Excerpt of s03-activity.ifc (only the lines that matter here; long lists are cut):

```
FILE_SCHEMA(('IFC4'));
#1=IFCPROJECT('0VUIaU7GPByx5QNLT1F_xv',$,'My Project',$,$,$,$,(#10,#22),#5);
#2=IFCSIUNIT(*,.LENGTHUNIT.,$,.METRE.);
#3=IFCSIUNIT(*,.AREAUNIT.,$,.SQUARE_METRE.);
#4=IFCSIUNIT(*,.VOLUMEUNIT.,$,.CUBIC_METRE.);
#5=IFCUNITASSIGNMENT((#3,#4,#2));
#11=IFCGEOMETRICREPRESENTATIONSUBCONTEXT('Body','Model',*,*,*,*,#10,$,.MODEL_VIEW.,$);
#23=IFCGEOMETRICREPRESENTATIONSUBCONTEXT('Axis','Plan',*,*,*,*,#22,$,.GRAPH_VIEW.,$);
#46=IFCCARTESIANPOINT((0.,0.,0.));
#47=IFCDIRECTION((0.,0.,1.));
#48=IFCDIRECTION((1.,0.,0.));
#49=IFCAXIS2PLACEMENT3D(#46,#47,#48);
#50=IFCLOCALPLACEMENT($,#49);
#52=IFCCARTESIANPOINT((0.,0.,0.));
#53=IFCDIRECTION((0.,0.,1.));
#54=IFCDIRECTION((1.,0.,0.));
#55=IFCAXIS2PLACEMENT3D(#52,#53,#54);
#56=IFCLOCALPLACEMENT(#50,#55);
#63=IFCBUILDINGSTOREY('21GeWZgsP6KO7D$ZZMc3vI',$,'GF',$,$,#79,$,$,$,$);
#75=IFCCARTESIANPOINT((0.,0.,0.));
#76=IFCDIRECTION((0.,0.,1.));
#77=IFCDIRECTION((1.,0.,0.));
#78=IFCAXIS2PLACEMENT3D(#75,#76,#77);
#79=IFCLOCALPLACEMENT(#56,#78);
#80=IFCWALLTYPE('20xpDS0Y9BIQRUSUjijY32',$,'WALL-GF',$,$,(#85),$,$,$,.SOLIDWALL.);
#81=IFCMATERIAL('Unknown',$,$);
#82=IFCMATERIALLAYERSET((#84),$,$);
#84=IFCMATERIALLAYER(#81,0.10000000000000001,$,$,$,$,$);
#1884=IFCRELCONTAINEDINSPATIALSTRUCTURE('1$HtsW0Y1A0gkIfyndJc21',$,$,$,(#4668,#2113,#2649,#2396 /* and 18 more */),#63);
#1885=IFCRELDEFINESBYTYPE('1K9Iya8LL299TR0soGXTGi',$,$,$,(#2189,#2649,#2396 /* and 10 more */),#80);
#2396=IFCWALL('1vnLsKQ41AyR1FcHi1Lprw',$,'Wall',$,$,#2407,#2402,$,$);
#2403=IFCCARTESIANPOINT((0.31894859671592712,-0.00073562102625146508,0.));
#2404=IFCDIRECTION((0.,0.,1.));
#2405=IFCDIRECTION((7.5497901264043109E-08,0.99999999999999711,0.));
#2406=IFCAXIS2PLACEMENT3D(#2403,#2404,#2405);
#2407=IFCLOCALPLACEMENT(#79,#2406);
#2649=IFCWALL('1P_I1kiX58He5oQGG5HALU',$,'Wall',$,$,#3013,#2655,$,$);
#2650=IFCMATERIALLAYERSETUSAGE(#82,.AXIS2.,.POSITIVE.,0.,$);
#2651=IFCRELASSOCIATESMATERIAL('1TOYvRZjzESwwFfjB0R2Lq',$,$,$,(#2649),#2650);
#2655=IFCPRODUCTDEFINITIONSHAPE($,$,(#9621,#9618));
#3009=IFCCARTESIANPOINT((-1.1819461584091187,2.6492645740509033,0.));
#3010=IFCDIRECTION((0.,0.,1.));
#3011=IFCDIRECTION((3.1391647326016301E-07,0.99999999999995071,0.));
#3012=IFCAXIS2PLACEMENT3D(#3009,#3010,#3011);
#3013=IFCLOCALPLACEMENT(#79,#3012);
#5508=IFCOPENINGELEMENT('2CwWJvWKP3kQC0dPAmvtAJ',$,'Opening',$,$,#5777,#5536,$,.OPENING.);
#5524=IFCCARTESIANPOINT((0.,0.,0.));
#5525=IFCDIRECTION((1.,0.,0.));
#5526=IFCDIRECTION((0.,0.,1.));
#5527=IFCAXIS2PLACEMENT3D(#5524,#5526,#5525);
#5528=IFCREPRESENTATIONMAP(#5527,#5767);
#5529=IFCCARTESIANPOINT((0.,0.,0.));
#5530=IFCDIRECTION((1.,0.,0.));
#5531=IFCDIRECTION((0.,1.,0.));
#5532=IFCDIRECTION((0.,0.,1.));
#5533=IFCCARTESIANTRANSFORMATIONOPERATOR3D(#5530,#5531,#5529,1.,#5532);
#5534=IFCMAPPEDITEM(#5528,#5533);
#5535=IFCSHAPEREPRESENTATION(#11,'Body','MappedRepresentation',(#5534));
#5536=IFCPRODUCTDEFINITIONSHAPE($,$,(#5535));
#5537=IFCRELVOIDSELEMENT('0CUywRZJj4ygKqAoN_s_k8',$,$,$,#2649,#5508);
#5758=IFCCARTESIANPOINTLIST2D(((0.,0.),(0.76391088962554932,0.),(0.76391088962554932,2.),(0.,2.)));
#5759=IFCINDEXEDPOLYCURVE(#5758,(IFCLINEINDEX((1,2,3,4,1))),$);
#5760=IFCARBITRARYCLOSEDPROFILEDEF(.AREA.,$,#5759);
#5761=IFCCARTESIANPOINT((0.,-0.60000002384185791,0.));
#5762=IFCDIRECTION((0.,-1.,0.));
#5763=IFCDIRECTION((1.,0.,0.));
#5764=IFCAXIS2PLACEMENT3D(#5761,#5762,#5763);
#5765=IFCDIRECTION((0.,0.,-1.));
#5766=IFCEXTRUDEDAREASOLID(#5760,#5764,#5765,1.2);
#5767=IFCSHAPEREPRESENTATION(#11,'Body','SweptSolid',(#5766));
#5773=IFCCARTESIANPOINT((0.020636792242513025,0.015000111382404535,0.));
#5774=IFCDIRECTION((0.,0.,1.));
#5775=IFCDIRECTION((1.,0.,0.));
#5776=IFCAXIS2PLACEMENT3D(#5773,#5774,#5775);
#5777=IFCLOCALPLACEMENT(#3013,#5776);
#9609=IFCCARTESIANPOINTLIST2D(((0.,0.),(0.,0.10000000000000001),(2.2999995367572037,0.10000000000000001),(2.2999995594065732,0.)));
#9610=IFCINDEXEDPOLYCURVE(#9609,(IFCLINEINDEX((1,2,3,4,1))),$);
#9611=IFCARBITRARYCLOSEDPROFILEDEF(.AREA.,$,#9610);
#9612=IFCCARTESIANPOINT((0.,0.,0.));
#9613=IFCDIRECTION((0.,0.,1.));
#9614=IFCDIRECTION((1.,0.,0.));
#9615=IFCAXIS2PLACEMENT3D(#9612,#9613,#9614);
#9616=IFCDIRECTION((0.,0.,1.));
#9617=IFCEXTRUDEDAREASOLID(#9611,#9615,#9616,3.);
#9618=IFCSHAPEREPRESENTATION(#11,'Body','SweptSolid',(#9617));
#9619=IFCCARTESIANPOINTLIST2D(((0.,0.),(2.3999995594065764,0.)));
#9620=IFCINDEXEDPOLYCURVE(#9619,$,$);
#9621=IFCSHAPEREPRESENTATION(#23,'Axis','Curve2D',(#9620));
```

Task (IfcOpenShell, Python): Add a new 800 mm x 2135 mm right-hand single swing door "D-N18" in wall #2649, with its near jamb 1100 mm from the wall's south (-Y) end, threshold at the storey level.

```python
import numpy as np
import ifcopenshell
import ifcopenshell.api.feature
import ifcopenshell.api.geometry
import ifcopenshell.api.root
import ifcopenshell.api.spatial
import ifcopenshell.geom
import ifcopenshell.util.element
import ifcopenshell.util.placement
import ifcopenshell.util.representation
import ifcopenshell.util.shape
import ifcopenshell.util.unit

model = ifcopenshell.open("s03-activity.ifc")
unit_scale = ifcopenshell.util.unit.calculate_unit_scale(model)
settings = ifcopenshell.geom.settings()


def volume(element):
    """Net volume in cubic metres, openings subtracted."""
    shape = ifcopenshell.geom.create_shape(settings, element)
    return ifcopenshell.util.shape.get_volume(shape.geometry)


wall = model.by_guid("1P_I1kiX58He5oQGG5HALU")
storey = ifcopenshell.util.element.get_container(wall, ifc_class="IfcBuildingStorey")
context = ifcopenshell.util.representation.get_context(model, "Model", "Body", "MODEL_VIEW")
before = volume(wall)

width, height, from_end, sill = 0.8, 2.135, 1.1, 0.0  # metres

# The wall runs along its own X axis, and the end named is its -X end.
wall_shape = ifcopenshell.geom.create_shape(settings, wall)
x, y, z = ifcopenshell.util.shape.get_vertices(wall_shape.geometry).T
start = x.min() + from_end
face, thickness = float(y.min()), float(y.max() - y.min())
wall_matrix = ifcopenshell.util.placement.get_local_placement(wall.ObjectPlacement)
level = ifcopenshell.util.placement.get_local_placement(storey.ObjectPlacement)[2, 3]


def in_wall(x, y):
    """Placement at x, y metres in the wall's axes, at sill height."""
    matrix = wall_matrix.copy()
    matrix[:, 3] = wall_matrix @ np.array([x / unit_scale, y / unit_scale, 0.0, 1.0])
    matrix[2, 3] = level + sill / unit_scale
    return matrix


# Opening: a box that overshoots both wall faces by 50 mm.
opening = ifcopenshell.api.root.create_entity(model, ifc_class="IfcOpeningElement", predefined_type="OPENING")
box = ifcopenshell.api.geometry.add_wall_representation(
    model, context=context, length=width, height=height, thickness=thickness + 0.1
)
ifcopenshell.api.geometry.assign_representation(model, product=opening, representation=box)
ifcopenshell.api.geometry.edit_object_placement(model, product=opening, matrix=in_wall(start, face - 0.05), is_si=False)
ifcopenshell.api.feature.add_feature(model, feature=opening, element=wall)

door = ifcopenshell.api.root.create_entity(model, ifc_class="IfcDoor", name="D-N18", predefined_type="DOOR")
door.OverallWidth, door.OverallHeight = width / unit_scale, height / unit_scale
door.OperationType = "SINGLE_SWING_RIGHT"
body = ifcopenshell.api.geometry.add_door_representation(
    model,
    context=context,
    overall_width=door.OverallWidth,
    overall_height=door.OverallHeight,
    operation_type="SINGLE_SWING_RIGHT",
    lining_properties={"LiningDepth": thickness / unit_scale, "ThresholdDepth": thickness / unit_scale},
)
ifcopenshell.api.geometry.assign_representation(model, product=door, representation=body)
ifcopenshell.api.spatial.assign_container(model, products=[door], relating_structure=storey)
ifcopenshell.api.feature.add_filling(model, opening=opening, element=door)

# The lining spans the wall, so the door starts at the wall face.
ifcopenshell.api.geometry.edit_object_placement(model, product=door, matrix=in_wall(start, face), is_si=False)

after = volume(wall)

print(f"wall volume {before:.3f} -> {after:.3f} m3")

model.write("s03-activity_rev.ifc")
```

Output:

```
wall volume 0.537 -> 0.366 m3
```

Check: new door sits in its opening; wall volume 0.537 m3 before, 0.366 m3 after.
